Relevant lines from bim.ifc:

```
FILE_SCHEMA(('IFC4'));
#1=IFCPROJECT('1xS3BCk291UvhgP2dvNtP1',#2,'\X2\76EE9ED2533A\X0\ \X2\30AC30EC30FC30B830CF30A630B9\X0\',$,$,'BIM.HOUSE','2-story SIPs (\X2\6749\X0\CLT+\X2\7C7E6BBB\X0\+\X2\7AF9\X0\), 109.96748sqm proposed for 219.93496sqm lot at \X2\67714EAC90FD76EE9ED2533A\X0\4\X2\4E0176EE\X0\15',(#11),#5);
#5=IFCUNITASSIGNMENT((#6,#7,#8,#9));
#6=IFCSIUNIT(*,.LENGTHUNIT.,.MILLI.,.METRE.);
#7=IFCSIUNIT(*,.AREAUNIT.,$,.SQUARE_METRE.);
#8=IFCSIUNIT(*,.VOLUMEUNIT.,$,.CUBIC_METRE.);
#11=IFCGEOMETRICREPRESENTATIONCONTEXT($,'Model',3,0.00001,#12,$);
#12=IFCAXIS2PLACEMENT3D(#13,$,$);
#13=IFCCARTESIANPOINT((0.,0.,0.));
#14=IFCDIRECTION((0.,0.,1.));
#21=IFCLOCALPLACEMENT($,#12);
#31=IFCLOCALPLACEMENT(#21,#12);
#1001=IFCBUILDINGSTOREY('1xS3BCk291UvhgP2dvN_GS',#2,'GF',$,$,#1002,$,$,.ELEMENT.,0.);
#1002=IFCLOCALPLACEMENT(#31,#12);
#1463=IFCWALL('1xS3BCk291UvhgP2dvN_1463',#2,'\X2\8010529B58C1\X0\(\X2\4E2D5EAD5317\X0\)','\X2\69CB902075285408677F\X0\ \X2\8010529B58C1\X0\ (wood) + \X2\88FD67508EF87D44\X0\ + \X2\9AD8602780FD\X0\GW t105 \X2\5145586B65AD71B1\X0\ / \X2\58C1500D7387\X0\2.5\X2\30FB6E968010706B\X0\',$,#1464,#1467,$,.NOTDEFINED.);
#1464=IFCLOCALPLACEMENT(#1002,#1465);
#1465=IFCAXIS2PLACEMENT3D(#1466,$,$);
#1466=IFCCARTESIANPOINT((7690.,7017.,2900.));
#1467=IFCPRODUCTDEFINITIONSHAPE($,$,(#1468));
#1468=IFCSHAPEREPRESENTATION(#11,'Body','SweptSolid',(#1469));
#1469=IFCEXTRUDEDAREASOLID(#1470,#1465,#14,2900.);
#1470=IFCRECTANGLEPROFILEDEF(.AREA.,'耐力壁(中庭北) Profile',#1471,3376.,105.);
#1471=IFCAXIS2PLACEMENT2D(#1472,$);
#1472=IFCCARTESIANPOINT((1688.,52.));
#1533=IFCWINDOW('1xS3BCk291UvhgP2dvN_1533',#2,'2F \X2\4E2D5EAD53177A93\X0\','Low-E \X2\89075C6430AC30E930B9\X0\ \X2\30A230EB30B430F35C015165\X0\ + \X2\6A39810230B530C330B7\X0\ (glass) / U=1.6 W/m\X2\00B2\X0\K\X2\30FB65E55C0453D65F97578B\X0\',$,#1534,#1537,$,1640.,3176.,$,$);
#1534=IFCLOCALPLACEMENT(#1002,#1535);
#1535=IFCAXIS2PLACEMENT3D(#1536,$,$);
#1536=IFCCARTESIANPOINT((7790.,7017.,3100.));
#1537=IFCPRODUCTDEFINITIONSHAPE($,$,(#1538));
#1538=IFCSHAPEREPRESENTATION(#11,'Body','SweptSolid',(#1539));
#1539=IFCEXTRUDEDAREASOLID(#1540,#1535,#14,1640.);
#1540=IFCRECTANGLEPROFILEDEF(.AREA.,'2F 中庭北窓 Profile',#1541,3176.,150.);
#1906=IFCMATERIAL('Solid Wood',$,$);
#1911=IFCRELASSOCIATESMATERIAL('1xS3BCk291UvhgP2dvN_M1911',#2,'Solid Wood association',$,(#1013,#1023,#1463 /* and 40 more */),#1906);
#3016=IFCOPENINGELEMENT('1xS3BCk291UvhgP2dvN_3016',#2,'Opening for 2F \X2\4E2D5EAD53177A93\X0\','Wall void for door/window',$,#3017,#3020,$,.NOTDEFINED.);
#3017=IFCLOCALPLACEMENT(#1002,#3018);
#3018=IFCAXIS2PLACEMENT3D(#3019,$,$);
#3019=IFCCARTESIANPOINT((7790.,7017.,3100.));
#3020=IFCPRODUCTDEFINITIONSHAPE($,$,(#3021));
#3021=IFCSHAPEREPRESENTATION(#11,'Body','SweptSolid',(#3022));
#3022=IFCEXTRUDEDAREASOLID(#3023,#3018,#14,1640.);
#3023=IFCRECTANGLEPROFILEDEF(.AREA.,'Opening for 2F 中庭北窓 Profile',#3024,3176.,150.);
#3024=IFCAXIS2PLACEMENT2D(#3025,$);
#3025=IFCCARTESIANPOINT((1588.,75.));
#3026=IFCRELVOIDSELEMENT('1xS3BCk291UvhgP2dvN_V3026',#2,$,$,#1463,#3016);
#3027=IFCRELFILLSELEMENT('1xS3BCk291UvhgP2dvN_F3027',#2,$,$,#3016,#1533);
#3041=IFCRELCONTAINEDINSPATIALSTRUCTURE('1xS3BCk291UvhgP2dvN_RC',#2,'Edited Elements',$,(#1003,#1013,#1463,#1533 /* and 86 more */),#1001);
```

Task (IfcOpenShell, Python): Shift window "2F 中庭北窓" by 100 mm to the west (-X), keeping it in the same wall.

```python
import ifcopenshell
import ifcopenshell.api.geometry
import ifcopenshell.util.placement

model = ifcopenshell.open("bim.ifc")

window = model.by_id(1533)
opening = window.FillsVoids[0].RelatingOpeningElement
wall = opening.VoidsElements[0].RelatingBuildingElement

wall_matrix = ifcopenshell.util.placement.get_local_placement(wall.ObjectPlacement)
shift = wall_matrix[:3, 0] * -100.0
before = ifcopenshell.util.placement.get_local_placement(window.ObjectPlacement)[:3, 3].copy()

# The window is not placed relative to its opening, so move both.
for product in (opening, window):
    matrix = ifcopenshell.util.placement.get_local_placement(product.ObjectPlacement)
    matrix[:3, 3] += shift
    ifcopenshell.api.geometry.edit_object_placement(model, product=product, matrix=matrix, is_si=False)

after = ifcopenshell.util.placement.get_local_placement(window.ObjectPlacement)[:3, 3]
print("window moved by", (after - before).round(3) + 0.0)

model.write("bim_v2.ifc")
```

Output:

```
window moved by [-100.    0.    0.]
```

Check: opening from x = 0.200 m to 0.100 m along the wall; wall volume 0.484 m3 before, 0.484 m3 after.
